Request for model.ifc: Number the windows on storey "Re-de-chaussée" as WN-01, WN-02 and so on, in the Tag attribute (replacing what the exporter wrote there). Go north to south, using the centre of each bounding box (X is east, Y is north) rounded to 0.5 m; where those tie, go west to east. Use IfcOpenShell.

First a look at what the model holds.

```python
import ifcopenshell
import ifcopenshell.util.element
import ifcopenshell.util.placement

model = ifcopenshell.open("model.ifc")
print(model.schema)
storey = next(s for s in model.by_type("IfcBuildingStorey") if s.Name == "Re-de-chaussée")
windows = [e for e in ifcopenshell.util.element.get_decomposition(storey) if e.is_a("IfcWindow")]
for e in sorted(windows, key=lambda e: e.id()):
    origin = ifcopenshell.util.placement.get_local_placement(e.ObjectPlacement)[:3, 3]
    print(e.id(), e.Tag, e.Name, origin.round(2) + 0.0, sep=" | ")
```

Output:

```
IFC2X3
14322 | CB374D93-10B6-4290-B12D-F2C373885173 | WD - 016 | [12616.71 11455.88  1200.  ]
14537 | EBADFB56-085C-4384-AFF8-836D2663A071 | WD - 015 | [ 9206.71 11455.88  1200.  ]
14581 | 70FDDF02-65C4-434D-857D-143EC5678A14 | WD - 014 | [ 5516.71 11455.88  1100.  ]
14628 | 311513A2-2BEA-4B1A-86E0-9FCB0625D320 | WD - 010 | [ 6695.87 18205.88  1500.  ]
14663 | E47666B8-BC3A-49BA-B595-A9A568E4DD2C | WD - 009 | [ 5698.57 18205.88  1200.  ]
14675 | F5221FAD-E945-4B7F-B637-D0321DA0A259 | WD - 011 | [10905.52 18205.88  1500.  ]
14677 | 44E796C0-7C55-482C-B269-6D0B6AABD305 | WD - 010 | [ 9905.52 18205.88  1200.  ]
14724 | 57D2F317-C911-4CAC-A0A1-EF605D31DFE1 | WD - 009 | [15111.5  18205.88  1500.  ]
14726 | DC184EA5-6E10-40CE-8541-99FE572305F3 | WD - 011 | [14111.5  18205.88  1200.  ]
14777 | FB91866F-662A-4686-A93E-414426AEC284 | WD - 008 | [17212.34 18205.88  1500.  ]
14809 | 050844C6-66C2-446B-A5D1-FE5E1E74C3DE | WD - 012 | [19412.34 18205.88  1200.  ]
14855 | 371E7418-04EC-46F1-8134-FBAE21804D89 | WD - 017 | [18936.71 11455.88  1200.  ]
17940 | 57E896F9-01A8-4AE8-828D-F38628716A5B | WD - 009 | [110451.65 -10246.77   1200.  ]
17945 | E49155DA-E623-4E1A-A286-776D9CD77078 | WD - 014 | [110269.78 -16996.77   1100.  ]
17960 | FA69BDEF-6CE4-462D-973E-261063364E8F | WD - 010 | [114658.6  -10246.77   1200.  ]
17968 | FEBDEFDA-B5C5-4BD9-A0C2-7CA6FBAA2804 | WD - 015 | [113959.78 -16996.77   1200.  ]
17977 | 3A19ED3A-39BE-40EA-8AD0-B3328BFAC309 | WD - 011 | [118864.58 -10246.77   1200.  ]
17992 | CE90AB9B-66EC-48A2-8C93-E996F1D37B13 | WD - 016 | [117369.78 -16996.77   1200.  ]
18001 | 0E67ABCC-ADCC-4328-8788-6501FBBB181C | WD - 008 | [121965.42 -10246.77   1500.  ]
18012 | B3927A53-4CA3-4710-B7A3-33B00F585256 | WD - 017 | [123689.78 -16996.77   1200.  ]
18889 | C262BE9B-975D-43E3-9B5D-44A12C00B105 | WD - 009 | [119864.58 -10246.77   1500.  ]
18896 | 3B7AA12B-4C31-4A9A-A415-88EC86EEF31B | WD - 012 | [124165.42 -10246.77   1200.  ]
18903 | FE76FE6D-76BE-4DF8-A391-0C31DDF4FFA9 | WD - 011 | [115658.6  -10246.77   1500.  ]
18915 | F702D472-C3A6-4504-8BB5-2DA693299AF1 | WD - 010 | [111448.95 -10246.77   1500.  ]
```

```python
import ifcopenshell
import ifcopenshell.geom
import ifcopenshell.util.element
import ifcopenshell.util.shape

model = ifcopenshell.open("model.ifc")
settings = ifcopenshell.geom.settings()
settings.set("use-world-coords", True)


def centre(element):
    shape = ifcopenshell.geom.create_shape(settings, element)
    return ifcopenshell.util.shape.get_bbox_centroid(shape.geometry)


storey = next(s for s in model.by_type("IfcBuildingStorey") if s.Name == "Re-de-chaussée")
windows = [e for e in ifcopenshell.util.element.get_decomposition(storey) if e.is_a("IfcWindow")]

# Insertion points can sit at a corner or the storey origin, so sort by the geometry (in metres).
centres = {e: centre(e) for e in windows}
windows.sort(key=lambda e: (-round(centres[e][1] / 0.5), centres[e][0]))

for i, e in enumerate(windows, start=1):
    number = f"WN-{i:02d}"
    e.Tag = number
    print(e.id(), number)

model.write("model_updated.ifc")
```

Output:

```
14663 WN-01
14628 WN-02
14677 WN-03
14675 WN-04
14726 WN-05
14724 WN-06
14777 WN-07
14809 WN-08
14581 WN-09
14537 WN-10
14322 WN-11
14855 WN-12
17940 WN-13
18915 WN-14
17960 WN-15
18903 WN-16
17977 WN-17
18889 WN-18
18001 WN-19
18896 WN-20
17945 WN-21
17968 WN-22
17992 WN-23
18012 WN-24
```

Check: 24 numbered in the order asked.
